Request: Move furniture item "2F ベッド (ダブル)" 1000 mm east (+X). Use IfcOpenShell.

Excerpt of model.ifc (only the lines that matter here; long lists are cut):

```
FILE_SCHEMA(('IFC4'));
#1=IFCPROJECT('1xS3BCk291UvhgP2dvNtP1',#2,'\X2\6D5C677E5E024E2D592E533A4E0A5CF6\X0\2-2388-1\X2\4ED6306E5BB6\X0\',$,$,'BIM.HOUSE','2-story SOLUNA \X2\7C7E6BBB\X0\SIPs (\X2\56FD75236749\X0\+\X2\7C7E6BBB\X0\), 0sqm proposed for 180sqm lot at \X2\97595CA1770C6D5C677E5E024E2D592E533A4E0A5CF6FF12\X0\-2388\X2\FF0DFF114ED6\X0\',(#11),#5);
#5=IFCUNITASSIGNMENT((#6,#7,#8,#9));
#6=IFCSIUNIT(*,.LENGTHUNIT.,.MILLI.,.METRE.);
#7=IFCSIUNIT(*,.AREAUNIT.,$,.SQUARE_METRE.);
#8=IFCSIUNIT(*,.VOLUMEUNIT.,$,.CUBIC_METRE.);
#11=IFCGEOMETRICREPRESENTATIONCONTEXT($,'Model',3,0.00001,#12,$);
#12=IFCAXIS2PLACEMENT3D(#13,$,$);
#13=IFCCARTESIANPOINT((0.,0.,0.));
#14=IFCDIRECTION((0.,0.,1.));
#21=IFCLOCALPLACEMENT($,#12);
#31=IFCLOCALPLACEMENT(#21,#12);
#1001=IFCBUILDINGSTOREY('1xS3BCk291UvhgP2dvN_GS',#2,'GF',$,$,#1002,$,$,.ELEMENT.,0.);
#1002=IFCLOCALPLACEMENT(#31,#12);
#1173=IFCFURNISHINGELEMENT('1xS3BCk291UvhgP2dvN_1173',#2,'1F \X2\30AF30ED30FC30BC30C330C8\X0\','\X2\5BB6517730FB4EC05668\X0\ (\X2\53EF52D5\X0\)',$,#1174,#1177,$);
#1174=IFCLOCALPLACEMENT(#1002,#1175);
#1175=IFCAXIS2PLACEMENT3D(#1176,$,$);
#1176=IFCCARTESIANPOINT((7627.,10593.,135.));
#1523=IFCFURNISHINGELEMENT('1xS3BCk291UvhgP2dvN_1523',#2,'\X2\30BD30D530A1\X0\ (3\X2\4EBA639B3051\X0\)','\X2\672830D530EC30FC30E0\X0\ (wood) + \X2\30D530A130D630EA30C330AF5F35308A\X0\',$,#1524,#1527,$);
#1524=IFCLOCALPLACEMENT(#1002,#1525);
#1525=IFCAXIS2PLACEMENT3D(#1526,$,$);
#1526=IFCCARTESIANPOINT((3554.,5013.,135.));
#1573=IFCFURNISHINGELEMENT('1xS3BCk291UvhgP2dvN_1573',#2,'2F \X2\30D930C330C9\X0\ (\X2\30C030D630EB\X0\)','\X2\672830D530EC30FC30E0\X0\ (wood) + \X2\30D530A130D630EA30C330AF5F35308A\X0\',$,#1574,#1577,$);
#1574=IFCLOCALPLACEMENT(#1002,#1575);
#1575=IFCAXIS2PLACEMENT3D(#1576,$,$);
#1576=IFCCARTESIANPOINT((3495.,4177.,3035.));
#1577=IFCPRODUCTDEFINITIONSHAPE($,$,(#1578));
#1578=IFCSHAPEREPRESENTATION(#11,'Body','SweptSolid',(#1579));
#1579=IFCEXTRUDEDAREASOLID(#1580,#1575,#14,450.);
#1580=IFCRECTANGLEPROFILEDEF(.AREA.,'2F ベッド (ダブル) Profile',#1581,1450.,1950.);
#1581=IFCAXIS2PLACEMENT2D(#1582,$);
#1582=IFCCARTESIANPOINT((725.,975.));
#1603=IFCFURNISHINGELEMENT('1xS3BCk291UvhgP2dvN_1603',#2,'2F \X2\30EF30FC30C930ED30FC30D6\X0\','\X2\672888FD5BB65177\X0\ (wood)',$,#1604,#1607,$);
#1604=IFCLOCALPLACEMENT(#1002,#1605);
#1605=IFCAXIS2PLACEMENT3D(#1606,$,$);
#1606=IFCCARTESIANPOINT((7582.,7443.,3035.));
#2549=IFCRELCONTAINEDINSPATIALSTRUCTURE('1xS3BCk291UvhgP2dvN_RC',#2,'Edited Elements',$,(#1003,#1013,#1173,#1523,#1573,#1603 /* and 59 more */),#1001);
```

```python
import ifcopenshell
import ifcopenshell.api.geometry
import ifcopenshell.util.placement

model = ifcopenshell.open("model.ifc")

item = model.by_id(1573)
matrix = ifcopenshell.util.placement.get_local_placement(item.ObjectPlacement)
matrix[0, 3] += 1000.0
ifcopenshell.api.geometry.edit_object_placement(model, product=item, matrix=matrix, is_si=False)

print(ifcopenshell.util.placement.get_local_placement(item.ObjectPlacement).round(3) + 0.0)

model.write("model_v2.ifc")
```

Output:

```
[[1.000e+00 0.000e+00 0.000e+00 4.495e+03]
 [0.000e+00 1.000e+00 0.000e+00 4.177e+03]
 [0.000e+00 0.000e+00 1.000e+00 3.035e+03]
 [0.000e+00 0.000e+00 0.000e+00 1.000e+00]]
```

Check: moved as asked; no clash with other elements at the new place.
